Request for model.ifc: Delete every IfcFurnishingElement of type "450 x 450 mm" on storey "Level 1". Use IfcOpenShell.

First a look at what the model holds.

```python
import ifcopenshell
import ifcopenshell.util.element

model = ifcopenshell.open("model.ifc")
print(model.schema)
storey = next(s for s in model.by_type("IfcBuildingStorey") if s.Name == "Level 1")
furniture = [e for e in ifcopenshell.util.element.get_decomposition(storey) if e.is_a("IfcFurnishingElement")]
seen = {}
for e in furniture:
    element_type = ifcopenshell.util.element.get_type(e)
    name = element_type.Name if element_type not in (None, e) else None
    seen[name] = seen.get(name, 0) + 1
for name, count in sorted(seen.items(), key=str):
    print(count, "x", name)
```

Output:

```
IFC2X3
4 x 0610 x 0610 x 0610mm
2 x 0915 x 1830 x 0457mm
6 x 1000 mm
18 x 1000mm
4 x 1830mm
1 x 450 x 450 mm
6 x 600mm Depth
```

```python
import ifcopenshell
import ifcopenshell.api.root
import ifcopenshell.util.element

model = ifcopenshell.open("model.ifc")

storey = next(s for s in model.by_type("IfcBuildingStorey") if s.Name == "Level 1")
furniture = [e for e in ifcopenshell.util.element.get_decomposition(storey) if e.is_a("IfcFurnishingElement")]
targets = [e for e in furniture if (t := ifcopenshell.util.element.get_type(e)) not in (None, e) and t.Name == "450 x 450 mm"]

for e in targets:
    ifcopenshell.api.root.remove_product(model, product=e)
print(len(targets), "removed")

model.write("model_edited.ifc")
```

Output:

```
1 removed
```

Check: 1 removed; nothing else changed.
